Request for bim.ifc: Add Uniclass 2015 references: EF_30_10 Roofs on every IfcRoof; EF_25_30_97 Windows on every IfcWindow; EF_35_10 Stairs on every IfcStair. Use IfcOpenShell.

First a look at what the model holds.

```python
import ifcopenshell

model = ifcopenshell.open("bim.ifc")
print(model.schema)
print("classifications:", [c.Name for c in model.by_type("IfcClassification")])
for ifc_class in ("IfcDoor", "IfcRoof", "IfcStair", "IfcWall", "IfcWindow"):
    print(ifc_class, len(model.by_type(ifc_class)))
```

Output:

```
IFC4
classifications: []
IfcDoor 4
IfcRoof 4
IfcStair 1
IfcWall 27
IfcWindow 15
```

```python
import ifcopenshell
import ifcopenshell.api.classification

model = ifcopenshell.open("bim.ifc")

system = ifcopenshell.api.classification.add_classification(model, classification="Uniclass 2015")

codes = {
    "IfcRoof": ("EF_30_10", "Roofs"),
    "IfcWindow": ("EF_25_30_97", "Windows"),
    "IfcStair": ("EF_35_10", "Stairs"),
}
for ifc_class, (code, name) in codes.items():
    products = model.by_type(ifc_class)
    ifcopenshell.api.classification.add_reference(
        model, products=products, classification=system, identification=code, name=name
    )
    print(code, len(products))

model.write("bim_edited.ifc")
```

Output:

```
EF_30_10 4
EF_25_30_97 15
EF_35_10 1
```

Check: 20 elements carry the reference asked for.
